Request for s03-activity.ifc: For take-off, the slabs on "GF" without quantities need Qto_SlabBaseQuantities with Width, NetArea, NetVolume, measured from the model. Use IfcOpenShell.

First a look at what the model holds.

```python
import ifcopenshell
import ifcopenshell.util.element
import ifcopenshell.util.unit

model = ifcopenshell.open("s03-activity.ifc")
print(model.schema)
for unit_type in ("LENGTHUNIT", "AREAUNIT", "VOLUMEUNIT"):
    print(unit_type, ifcopenshell.util.unit.calculate_unit_scale(model, unit_type))
storey = next(s for s in model.by_type("IfcBuildingStorey") if s.Name == "GF")
slabs = [e for e in ifcopenshell.util.element.get_decomposition(storey) if e.is_a("IfcSlab")]
for e in sorted(slabs, key=lambda e: e.id()):
    print(e.id(), e.is_a(), e.Name, list(ifcopenshell.util.element.get_psets(e, qtos_only=True)), sep=" | ")
```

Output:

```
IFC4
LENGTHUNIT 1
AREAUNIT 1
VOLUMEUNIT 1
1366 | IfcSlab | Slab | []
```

```python
import ifcopenshell
import ifcopenshell.api.pset
import ifcopenshell.geom
import ifcopenshell.util.element
import ifcopenshell.util.shape
import ifcopenshell.util.unit

model = ifcopenshell.open("s03-activity.ifc")
unit_scale = ifcopenshell.util.unit.calculate_unit_scale(model)
area_scale = ifcopenshell.util.unit.calculate_unit_scale(model, "AREAUNIT")
volume_scale = ifcopenshell.util.unit.calculate_unit_scale(model, "VOLUMEUNIT")
settings = ifcopenshell.geom.settings()

storey = next(s for s in model.by_type("IfcBuildingStorey") if s.Name == "GF")
slabs = [e for e in ifcopenshell.util.element.get_decomposition(storey) if e.is_a("IfcSlab")]

for e in sorted(slabs, key=lambda e: e.id()):
    if ifcopenshell.util.element.get_psets(e, qtos_only=True, should_inherit=False):
        continue
    # Geometry comes back in metres, in the element's own axes.
    shape = ifcopenshell.geom.create_shape(settings, e)
    values = {
        "Width": ifcopenshell.util.shape.get_z(shape.geometry) / unit_scale,
        "NetArea": ifcopenshell.util.shape.get_footprint_area(shape.geometry) / area_scale,
        "NetVolume": ifcopenshell.util.shape.get_volume(shape.geometry) / volume_scale,
    }
    qto = ifcopenshell.api.pset.add_qto(model, product=e, name="Qto_SlabBaseQuantities")
    ifcopenshell.api.pset.edit_qto(model, qto=qto, properties=values)
    print(e.id(), {k: round(v, 3) for k, v in values.items()})

model.write("s03-activity_rev.ifc")
```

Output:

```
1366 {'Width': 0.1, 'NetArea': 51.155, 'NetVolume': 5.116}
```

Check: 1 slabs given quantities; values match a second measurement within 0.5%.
